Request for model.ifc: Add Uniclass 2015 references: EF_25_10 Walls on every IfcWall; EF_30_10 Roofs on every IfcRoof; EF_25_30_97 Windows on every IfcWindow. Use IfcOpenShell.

First a look at what the model holds.

```python
import ifcopenshell

model = ifcopenshell.open("model.ifc")
print(model.schema)
print("classifications:", [c.Name for c in model.by_type("IfcClassification")])
for ifc_class in ("IfcDoor", "IfcRoof", "IfcStair", "IfcWall", "IfcWindow"):
    print(ifc_class, len(model.by_type(ifc_class)))
```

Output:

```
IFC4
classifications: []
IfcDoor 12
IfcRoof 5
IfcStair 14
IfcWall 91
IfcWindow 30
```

```python
import ifcopenshell
import ifcopenshell.api.classification

model = ifcopenshell.open("model.ifc")

system = ifcopenshell.api.classification.add_classification(model, classification="Uniclass 2015")

codes = {
    "IfcWall": ("EF_25_10", "Walls"),
    "IfcRoof": ("EF_30_10", "Roofs"),
    "IfcWindow": ("EF_25_30_97", "Windows"),
}
for ifc_class, (code, name) in codes.items():
    products = model.by_type(ifc_class)
    ifcopenshell.api.classification.add_reference(
        model, products=products, classification=system, identification=code, name=name
    )
    print(code, len(products))

model.write("model-out.ifc")
```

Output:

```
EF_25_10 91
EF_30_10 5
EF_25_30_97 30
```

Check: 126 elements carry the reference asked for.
